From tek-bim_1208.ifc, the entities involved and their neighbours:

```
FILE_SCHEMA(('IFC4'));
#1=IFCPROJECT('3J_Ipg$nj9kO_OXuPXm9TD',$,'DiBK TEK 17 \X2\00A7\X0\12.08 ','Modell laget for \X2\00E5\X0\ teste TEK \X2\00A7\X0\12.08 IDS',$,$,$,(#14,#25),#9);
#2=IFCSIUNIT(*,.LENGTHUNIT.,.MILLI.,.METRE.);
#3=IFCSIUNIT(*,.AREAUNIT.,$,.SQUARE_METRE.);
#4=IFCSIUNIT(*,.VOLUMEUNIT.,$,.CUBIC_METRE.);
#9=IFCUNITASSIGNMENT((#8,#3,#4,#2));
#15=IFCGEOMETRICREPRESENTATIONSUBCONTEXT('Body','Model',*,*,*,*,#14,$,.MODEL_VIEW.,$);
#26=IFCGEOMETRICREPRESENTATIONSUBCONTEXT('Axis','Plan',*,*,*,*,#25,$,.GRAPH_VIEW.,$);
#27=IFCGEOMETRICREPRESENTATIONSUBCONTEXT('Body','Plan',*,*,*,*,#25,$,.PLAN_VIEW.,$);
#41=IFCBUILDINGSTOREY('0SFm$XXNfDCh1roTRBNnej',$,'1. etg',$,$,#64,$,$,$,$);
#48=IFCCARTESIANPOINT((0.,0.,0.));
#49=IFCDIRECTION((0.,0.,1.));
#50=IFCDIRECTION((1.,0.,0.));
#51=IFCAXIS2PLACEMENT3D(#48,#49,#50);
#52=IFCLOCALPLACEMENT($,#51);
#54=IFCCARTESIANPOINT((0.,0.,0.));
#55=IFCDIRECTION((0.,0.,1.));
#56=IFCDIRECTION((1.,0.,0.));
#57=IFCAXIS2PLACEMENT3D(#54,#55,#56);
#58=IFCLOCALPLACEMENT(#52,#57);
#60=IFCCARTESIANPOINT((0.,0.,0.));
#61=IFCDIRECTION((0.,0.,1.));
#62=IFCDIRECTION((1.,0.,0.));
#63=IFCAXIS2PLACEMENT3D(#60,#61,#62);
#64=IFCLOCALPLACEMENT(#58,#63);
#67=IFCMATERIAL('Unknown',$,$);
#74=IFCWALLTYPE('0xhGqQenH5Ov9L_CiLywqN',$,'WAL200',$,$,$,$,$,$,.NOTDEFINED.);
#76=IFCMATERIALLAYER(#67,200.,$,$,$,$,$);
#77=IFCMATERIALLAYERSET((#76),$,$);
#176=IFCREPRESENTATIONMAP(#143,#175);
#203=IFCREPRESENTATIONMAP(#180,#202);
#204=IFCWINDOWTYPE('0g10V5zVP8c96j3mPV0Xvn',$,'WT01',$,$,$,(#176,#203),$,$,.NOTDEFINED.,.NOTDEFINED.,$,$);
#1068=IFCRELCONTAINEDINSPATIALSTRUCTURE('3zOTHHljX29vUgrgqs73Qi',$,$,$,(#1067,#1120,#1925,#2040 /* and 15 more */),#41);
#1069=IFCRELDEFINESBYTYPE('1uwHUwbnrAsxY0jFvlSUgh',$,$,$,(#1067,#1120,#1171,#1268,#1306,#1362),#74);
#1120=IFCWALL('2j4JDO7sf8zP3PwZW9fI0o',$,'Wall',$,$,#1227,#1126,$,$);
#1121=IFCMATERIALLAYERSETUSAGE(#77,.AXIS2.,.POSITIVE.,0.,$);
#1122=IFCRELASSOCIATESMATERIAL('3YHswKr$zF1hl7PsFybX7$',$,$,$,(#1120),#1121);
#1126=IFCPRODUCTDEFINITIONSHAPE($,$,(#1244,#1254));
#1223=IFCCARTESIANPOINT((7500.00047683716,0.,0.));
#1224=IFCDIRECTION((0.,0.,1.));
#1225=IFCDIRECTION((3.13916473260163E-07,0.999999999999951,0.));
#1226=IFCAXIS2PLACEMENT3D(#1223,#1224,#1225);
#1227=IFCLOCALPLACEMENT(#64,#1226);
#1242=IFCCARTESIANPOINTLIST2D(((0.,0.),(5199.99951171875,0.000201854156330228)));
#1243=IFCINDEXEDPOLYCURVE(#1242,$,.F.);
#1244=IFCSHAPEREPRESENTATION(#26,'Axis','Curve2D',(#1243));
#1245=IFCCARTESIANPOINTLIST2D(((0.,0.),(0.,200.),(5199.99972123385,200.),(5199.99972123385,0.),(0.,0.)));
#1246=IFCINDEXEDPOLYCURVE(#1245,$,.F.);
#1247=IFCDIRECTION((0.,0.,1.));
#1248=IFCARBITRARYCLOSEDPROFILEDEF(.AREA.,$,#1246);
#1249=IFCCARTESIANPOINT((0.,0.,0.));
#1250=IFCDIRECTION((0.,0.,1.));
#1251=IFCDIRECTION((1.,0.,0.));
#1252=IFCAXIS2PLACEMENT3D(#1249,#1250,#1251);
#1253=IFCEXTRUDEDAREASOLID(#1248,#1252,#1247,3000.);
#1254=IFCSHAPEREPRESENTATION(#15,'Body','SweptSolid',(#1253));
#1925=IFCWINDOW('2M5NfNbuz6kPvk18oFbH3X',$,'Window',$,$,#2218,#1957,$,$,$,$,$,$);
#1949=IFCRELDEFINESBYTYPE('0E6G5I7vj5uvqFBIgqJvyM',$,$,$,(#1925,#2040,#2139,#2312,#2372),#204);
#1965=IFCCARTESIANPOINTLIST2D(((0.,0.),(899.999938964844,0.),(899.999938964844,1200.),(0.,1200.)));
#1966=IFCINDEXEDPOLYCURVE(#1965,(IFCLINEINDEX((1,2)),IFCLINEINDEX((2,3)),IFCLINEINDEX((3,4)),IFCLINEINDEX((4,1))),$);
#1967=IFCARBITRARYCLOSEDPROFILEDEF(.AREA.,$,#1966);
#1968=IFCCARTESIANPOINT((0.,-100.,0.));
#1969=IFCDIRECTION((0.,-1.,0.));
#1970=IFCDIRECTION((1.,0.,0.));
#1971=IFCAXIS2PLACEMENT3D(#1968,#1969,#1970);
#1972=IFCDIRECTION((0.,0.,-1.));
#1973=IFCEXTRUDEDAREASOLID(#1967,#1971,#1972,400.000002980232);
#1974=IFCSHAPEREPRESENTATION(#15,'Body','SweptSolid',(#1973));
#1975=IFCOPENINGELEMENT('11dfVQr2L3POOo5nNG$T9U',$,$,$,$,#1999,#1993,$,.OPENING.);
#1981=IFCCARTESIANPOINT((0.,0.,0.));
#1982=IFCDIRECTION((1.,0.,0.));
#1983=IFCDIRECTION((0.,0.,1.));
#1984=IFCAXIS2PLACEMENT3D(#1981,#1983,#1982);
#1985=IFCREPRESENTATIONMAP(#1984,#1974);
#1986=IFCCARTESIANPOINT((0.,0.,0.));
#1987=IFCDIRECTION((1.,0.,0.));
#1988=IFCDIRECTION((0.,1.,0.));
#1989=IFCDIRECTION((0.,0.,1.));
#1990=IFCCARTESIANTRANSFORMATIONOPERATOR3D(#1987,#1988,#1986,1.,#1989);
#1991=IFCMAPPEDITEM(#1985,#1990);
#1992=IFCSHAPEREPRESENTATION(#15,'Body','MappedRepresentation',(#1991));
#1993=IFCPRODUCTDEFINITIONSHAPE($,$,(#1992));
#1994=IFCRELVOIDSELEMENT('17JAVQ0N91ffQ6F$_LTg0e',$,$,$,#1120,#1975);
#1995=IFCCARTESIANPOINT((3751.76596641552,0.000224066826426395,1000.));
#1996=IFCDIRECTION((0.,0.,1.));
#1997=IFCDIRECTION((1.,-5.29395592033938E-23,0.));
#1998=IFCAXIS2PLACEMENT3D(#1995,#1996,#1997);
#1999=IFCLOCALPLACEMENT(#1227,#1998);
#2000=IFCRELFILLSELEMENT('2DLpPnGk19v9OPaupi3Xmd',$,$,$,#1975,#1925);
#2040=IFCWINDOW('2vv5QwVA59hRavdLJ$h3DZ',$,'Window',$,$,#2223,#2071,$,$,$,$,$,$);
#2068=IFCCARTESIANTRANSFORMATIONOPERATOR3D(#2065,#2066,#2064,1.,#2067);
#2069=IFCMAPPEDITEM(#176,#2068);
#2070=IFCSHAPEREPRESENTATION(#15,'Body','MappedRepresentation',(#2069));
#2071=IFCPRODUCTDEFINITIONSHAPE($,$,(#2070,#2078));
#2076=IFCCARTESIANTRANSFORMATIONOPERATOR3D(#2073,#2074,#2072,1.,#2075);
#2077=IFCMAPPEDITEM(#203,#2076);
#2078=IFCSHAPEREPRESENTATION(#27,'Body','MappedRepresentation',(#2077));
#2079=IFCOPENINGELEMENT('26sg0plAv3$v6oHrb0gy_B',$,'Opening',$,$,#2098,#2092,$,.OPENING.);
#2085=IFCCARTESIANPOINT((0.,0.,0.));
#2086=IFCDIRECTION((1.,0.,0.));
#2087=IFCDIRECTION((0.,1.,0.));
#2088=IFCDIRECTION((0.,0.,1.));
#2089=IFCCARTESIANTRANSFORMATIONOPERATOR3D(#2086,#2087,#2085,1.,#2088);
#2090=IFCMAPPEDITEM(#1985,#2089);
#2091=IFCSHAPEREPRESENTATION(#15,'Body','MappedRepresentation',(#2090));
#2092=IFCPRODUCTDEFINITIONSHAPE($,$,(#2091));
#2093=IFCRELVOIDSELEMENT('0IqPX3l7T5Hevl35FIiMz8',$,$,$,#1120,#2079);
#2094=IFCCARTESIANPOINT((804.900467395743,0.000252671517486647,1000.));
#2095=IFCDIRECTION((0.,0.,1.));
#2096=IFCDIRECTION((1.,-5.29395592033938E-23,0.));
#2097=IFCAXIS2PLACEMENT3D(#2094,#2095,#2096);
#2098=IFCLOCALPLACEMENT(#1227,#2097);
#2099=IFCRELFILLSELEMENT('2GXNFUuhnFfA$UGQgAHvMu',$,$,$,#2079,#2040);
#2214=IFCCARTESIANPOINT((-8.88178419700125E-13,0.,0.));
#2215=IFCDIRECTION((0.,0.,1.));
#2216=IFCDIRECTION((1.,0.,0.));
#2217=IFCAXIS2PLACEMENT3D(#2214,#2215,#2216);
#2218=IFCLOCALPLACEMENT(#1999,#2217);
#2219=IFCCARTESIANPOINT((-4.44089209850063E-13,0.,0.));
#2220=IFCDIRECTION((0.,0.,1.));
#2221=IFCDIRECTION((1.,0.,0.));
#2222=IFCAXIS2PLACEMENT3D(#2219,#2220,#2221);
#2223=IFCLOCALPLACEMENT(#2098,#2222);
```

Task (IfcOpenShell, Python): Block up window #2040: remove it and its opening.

```python
import ifcopenshell
import ifcopenshell.api.feature
import ifcopenshell.api.root
import ifcopenshell.geom
import ifcopenshell.util.shape

model = ifcopenshell.open("tek-bim_1208.ifc")
settings = ifcopenshell.geom.settings()


def volume(element):
    """Net volume in cubic metres, openings subtracted."""
    shape = ifcopenshell.geom.create_shape(settings, element)
    return ifcopenshell.util.shape.get_volume(shape.geometry)


window = model.by_id(2040)
opening = window.FillsVoids[0].RelatingOpeningElement
wall = opening.VoidsElements[0].RelatingBuildingElement
before = volume(wall)

ifcopenshell.api.root.remove_product(model, product=window)
ifcopenshell.api.feature.remove_feature(model, feature=opening)

after = volume(wall)

print(f"wall volume {before:.3f} -> {after:.3f} m3")

model.write("tek-bim_1208-out.ifc")
```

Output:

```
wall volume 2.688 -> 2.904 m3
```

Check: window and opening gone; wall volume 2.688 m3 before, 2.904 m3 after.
